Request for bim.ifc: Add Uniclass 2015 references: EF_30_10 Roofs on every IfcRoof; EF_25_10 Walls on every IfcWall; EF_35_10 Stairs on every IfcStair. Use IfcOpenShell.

First a look at what the model holds.

```python
import ifcopenshell

model = ifcopenshell.open("bim.ifc")
print(model.schema)
print("classifications:", [c.Name for c in model.by_type("IfcClassification")])
for ifc_class in ("IfcDoor", "IfcRoof", "IfcStair", "IfcWall", "IfcWindow"):
    print(ifc_class, len(model.by_type(ifc_class)))
```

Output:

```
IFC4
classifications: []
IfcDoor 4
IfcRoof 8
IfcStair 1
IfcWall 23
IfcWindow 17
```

```python
import ifcopenshell
import ifcopenshell.api.classification

model = ifcopenshell.open("bim.ifc")

system = ifcopenshell.api.classification.add_classification(model, classification="Uniclass 2015")

codes = {
    "IfcRoof": ("EF_30_10", "Roofs"),
    "IfcWall": ("EF_25_10", "Walls"),
    "IfcStair": ("EF_35_10", "Stairs"),
}
for ifc_class, (code, name) in codes.items():
    products = model.by_type(ifc_class)
    ifcopenshell.api.classification.add_reference(
        model, products=products, classification=system, identification=code, name=name
    )
    print(code, len(products))

model.write("bim_rev.ifc")
```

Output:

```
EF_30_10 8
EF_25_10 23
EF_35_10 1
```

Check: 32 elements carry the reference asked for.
